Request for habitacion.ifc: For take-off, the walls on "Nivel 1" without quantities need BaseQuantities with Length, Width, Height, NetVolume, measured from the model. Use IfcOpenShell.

First a look at what the model holds.

```python
import ifcopenshell
import ifcopenshell.util.element
import ifcopenshell.util.unit

model = ifcopenshell.open("habitacion.ifc")
print(model.schema)
for unit_type in ("LENGTHUNIT", "AREAUNIT", "VOLUMEUNIT"):
    print(unit_type, ifcopenshell.util.unit.calculate_unit_scale(model, unit_type))
storey = next(s for s in model.by_type("IfcBuildingStorey") if s.Name == "Nivel 1")
walls = [e for e in ifcopenshell.util.element.get_decomposition(storey) if e.is_a("IfcWall")]
for e in sorted(walls, key=lambda e: e.id()):
    print(e.id(), e.is_a(), e.Name, list(ifcopenshell.util.element.get_psets(e, qtos_only=True)), sep=" | ")
```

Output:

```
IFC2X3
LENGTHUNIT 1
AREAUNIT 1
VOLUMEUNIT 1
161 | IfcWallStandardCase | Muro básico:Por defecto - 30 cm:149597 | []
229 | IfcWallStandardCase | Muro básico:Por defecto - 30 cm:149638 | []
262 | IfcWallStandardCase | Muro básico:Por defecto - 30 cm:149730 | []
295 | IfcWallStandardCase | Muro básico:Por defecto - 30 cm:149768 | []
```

```python
import ifcopenshell
import ifcopenshell.api.pset
import ifcopenshell.geom
import ifcopenshell.util.element
import ifcopenshell.util.shape
import ifcopenshell.util.unit

model = ifcopenshell.open("habitacion.ifc")
unit_scale = ifcopenshell.util.unit.calculate_unit_scale(model)
volume_scale = ifcopenshell.util.unit.calculate_unit_scale(model, "VOLUMEUNIT")
settings = ifcopenshell.geom.settings()

storey = next(s for s in model.by_type("IfcBuildingStorey") if s.Name == "Nivel 1")
walls = [e for e in ifcopenshell.util.element.get_decomposition(storey) if e.is_a("IfcWall")]

for e in sorted(walls, key=lambda e: e.id()):
    if ifcopenshell.util.element.get_psets(e, qtos_only=True, should_inherit=False):
        continue
    # Geometry comes back in metres, in the element's own axes.
    shape = ifcopenshell.geom.create_shape(settings, e)
    values = {
        "Length": ifcopenshell.util.shape.get_x(shape.geometry) / unit_scale,
        "Width": ifcopenshell.util.shape.get_y(shape.geometry) / unit_scale,
        "Height": ifcopenshell.util.shape.get_z(shape.geometry) / unit_scale,
        "NetVolume": ifcopenshell.util.shape.get_volume(shape.geometry) / volume_scale,
    }
    qto = ifcopenshell.api.pset.add_qto(model, product=e, name="BaseQuantities")
    ifcopenshell.api.pset.edit_qto(model, qto=qto, properties=values)
    print(e.id(), {k: round(v, 3) for k, v in values.items()})

model.write("habitacion_edited.ifc")
```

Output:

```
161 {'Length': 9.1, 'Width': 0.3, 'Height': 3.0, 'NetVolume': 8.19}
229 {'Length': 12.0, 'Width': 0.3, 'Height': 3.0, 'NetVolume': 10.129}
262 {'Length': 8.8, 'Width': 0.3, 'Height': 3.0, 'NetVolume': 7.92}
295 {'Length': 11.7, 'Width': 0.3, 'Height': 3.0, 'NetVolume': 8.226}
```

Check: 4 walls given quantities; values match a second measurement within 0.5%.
